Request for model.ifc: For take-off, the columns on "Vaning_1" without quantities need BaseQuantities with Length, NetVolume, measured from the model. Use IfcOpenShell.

First a look at what the model holds.

```python
import ifcopenshell
import ifcopenshell.util.element
import ifcopenshell.util.unit

model = ifcopenshell.open("model.ifc")
print(model.schema)
for unit_type in ("LENGTHUNIT", "AREAUNIT", "VOLUMEUNIT"):
    print(unit_type, ifcopenshell.util.unit.calculate_unit_scale(model, unit_type))
storey = next(s for s in model.by_type("IfcBuildingStorey") if s.Name == "Vaning_1")
columns = [e for e in ifcopenshell.util.element.get_decomposition(storey) if e.is_a("IfcColumn")]
for e in sorted(columns, key=lambda e: e.id()):
    print(e.id(), e.is_a(), e.Name, list(ifcopenshell.util.element.get_psets(e, qtos_only=True)), sep=" | ")
```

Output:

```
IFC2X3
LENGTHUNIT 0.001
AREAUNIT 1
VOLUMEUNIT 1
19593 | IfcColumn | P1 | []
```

```python
import ifcopenshell
import ifcopenshell.api.pset
import ifcopenshell.geom
import ifcopenshell.util.element
import ifcopenshell.util.shape
import ifcopenshell.util.unit

model = ifcopenshell.open("model.ifc")
unit_scale = ifcopenshell.util.unit.calculate_unit_scale(model)
volume_scale = ifcopenshell.util.unit.calculate_unit_scale(model, "VOLUMEUNIT")
settings = ifcopenshell.geom.settings()

storey = next(s for s in model.by_type("IfcBuildingStorey") if s.Name == "Vaning_1")
columns = [e for e in ifcopenshell.util.element.get_decomposition(storey) if e.is_a("IfcColumn")]

for e in sorted(columns, key=lambda e: e.id()):
    if ifcopenshell.util.element.get_psets(e, qtos_only=True, should_inherit=False):
        continue
    # Geometry comes back in metres, in the element's own axes.
    shape = ifcopenshell.geom.create_shape(settings, e)
    values = {
        "Length": ifcopenshell.util.shape.get_z(shape.geometry) / unit_scale,
        "NetVolume": ifcopenshell.util.shape.get_volume(shape.geometry) / volume_scale,
    }
    qto = ifcopenshell.api.pset.add_qto(model, product=e, name="BaseQuantities")
    ifcopenshell.api.pset.edit_qto(model, qto=qto, properties=values)
    print(e.id(), {k: round(v, 3) for k, v in values.items()})

model.write("model_v2.ifc")
```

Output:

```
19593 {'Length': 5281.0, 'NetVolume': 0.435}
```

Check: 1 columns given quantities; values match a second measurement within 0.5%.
